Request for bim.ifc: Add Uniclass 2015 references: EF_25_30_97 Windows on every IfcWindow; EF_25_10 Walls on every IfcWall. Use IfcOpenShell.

First a look at what the model holds.

```python
import ifcopenshell

model = ifcopenshell.open("bim.ifc")
print(model.schema)
print("classifications:", [c.Name for c in model.by_type("IfcClassification")])
for ifc_class in ("IfcDoor", "IfcRoof", "IfcStair", "IfcWall", "IfcWindow"):
    print(ifc_class, len(model.by_type(ifc_class)))
```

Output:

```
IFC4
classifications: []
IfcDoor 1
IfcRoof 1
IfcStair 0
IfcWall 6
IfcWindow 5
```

```python
import ifcopenshell
import ifcopenshell.api.classification

model = ifcopenshell.open("bim.ifc")

system = ifcopenshell.api.classification.add_classification(model, classification="Uniclass 2015")

codes = {
    "IfcWindow": ("EF_25_30_97", "Windows"),
    "IfcWall": ("EF_25_10", "Walls"),
}
for ifc_class, (code, name) in codes.items():
    products = model.by_type(ifc_class)
    ifcopenshell.api.classification.add_reference(
        model, products=products, classification=system, identification=code, name=name
    )
    print(code, len(products))

model.write("bim_rev.ifc")
```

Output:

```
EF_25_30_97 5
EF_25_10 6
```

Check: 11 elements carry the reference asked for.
